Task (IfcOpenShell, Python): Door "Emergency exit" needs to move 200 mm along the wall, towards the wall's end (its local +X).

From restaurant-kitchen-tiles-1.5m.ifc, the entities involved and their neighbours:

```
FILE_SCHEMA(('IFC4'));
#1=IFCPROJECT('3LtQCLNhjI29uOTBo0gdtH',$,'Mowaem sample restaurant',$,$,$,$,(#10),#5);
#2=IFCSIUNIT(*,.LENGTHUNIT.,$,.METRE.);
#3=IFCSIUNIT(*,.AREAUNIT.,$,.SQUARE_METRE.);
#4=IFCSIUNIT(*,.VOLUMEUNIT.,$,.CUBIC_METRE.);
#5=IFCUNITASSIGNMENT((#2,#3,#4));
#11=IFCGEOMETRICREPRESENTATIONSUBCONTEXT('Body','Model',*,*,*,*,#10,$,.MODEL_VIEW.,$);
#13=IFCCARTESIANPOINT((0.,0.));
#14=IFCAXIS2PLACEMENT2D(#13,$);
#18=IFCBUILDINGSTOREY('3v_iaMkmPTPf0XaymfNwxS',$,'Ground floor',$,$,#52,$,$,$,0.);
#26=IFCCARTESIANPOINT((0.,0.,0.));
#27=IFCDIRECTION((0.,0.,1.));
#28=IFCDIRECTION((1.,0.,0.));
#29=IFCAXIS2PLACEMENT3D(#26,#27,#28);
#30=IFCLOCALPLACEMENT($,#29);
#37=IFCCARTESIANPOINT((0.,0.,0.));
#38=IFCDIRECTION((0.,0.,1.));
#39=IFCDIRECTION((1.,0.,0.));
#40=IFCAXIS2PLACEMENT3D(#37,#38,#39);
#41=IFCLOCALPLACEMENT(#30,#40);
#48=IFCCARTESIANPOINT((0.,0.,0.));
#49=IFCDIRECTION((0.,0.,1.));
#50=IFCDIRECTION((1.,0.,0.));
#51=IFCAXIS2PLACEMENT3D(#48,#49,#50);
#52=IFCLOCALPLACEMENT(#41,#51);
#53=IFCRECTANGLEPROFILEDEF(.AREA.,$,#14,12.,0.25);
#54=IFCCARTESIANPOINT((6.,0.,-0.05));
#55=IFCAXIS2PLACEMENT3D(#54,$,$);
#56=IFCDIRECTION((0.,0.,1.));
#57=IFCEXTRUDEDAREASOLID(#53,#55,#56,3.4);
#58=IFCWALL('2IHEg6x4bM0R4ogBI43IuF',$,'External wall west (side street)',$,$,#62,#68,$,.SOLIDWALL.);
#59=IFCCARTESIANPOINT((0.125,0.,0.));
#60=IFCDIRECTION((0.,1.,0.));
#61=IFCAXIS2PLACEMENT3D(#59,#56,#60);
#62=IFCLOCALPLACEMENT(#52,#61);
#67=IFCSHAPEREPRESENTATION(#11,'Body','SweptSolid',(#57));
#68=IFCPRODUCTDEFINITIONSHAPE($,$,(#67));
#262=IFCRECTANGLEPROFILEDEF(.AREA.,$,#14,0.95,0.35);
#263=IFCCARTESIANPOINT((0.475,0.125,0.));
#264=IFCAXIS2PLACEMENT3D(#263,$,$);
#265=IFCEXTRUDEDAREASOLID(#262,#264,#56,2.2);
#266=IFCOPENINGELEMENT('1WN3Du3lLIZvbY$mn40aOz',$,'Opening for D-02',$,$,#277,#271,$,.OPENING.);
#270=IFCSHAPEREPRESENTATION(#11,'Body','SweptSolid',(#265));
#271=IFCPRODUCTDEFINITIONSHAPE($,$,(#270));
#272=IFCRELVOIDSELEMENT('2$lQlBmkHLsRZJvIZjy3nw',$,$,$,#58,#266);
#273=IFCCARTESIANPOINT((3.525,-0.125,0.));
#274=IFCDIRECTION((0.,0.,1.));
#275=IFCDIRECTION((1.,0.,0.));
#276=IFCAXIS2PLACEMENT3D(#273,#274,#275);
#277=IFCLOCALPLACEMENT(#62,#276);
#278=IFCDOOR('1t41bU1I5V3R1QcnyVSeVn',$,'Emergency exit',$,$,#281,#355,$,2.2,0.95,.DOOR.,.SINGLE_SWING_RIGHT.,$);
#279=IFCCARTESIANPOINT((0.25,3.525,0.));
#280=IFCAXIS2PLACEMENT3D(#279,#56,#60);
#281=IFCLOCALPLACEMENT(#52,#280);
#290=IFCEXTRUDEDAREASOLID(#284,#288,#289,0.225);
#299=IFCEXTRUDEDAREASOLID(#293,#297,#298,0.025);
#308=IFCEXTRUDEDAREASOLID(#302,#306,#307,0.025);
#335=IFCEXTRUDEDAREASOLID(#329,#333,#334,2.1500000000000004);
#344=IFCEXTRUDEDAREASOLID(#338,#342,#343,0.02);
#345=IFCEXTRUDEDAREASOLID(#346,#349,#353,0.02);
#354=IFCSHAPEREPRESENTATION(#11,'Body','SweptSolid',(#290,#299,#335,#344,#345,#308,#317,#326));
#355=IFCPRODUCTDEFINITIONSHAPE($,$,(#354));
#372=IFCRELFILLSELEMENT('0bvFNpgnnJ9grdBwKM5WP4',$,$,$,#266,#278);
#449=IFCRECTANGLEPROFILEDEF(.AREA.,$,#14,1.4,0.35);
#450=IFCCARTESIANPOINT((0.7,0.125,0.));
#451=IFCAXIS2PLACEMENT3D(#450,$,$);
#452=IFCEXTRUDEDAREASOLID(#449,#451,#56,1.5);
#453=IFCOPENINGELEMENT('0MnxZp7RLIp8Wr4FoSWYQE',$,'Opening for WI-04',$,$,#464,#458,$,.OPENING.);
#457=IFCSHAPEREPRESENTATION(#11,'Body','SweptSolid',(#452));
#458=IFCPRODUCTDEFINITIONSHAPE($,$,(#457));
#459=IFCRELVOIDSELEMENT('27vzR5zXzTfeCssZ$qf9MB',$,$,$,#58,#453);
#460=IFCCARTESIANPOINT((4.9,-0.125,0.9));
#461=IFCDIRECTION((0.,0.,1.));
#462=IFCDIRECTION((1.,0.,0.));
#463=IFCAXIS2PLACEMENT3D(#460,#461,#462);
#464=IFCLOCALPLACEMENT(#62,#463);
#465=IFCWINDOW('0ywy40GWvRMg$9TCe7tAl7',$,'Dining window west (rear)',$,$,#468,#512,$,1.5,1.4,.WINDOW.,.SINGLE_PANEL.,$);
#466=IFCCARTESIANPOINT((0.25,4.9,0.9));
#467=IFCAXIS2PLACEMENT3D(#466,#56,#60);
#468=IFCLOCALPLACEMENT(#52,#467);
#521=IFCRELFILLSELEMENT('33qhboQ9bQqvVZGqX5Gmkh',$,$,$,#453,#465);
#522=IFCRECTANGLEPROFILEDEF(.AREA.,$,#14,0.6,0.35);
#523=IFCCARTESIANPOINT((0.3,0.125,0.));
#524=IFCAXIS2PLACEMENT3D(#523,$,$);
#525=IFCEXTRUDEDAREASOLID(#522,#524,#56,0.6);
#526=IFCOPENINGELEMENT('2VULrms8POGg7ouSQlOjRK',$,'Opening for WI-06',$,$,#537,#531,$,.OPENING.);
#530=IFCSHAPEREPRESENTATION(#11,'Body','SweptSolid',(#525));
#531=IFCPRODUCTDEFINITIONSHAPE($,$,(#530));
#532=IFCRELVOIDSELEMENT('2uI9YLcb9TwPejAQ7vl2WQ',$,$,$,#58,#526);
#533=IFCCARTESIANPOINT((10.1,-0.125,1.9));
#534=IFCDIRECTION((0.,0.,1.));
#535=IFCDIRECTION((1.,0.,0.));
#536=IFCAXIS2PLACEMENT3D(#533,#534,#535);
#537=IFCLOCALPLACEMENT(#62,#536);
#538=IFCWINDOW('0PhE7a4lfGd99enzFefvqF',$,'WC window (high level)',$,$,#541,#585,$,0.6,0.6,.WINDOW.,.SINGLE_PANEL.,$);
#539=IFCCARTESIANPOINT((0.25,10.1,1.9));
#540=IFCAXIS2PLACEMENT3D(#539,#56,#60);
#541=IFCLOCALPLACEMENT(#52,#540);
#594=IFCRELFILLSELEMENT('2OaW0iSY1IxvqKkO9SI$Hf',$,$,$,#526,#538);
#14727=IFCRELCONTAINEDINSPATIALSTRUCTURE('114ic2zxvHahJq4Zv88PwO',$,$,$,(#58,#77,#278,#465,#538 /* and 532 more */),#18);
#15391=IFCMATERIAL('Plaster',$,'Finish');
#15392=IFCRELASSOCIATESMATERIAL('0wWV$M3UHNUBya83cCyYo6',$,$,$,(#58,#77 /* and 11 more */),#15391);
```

```python
import ifcopenshell
import ifcopenshell.api.geometry
import ifcopenshell.util.placement

model = ifcopenshell.open("restaurant-kitchen-tiles-1.5m.ifc")

door = model.by_guid("1t41bU1I5V3R1QcnyVSeVn")
opening = door.FillsVoids[0].RelatingOpeningElement
wall = opening.VoidsElements[0].RelatingBuildingElement

wall_matrix = ifcopenshell.util.placement.get_local_placement(wall.ObjectPlacement)
shift = wall_matrix[:3, 0] * 0.2
before = ifcopenshell.util.placement.get_local_placement(door.ObjectPlacement)[:3, 3].copy()

# The door is not placed relative to its opening, so move both.
for product in (opening, door):
    matrix = ifcopenshell.util.placement.get_local_placement(product.ObjectPlacement)
    matrix[:3, 3] += shift
    ifcopenshell.api.geometry.edit_object_placement(model, product=product, matrix=matrix, is_si=False)

after = ifcopenshell.util.placement.get_local_placement(door.ObjectPlacement)[:3, 3]
print("door moved by", (after - before).round(3) + 0.0)

model.write("restaurant-kitchen-tiles-1.5m_edited.ifc")
```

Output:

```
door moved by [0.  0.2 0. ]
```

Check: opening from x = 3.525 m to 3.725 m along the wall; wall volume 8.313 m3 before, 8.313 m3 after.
